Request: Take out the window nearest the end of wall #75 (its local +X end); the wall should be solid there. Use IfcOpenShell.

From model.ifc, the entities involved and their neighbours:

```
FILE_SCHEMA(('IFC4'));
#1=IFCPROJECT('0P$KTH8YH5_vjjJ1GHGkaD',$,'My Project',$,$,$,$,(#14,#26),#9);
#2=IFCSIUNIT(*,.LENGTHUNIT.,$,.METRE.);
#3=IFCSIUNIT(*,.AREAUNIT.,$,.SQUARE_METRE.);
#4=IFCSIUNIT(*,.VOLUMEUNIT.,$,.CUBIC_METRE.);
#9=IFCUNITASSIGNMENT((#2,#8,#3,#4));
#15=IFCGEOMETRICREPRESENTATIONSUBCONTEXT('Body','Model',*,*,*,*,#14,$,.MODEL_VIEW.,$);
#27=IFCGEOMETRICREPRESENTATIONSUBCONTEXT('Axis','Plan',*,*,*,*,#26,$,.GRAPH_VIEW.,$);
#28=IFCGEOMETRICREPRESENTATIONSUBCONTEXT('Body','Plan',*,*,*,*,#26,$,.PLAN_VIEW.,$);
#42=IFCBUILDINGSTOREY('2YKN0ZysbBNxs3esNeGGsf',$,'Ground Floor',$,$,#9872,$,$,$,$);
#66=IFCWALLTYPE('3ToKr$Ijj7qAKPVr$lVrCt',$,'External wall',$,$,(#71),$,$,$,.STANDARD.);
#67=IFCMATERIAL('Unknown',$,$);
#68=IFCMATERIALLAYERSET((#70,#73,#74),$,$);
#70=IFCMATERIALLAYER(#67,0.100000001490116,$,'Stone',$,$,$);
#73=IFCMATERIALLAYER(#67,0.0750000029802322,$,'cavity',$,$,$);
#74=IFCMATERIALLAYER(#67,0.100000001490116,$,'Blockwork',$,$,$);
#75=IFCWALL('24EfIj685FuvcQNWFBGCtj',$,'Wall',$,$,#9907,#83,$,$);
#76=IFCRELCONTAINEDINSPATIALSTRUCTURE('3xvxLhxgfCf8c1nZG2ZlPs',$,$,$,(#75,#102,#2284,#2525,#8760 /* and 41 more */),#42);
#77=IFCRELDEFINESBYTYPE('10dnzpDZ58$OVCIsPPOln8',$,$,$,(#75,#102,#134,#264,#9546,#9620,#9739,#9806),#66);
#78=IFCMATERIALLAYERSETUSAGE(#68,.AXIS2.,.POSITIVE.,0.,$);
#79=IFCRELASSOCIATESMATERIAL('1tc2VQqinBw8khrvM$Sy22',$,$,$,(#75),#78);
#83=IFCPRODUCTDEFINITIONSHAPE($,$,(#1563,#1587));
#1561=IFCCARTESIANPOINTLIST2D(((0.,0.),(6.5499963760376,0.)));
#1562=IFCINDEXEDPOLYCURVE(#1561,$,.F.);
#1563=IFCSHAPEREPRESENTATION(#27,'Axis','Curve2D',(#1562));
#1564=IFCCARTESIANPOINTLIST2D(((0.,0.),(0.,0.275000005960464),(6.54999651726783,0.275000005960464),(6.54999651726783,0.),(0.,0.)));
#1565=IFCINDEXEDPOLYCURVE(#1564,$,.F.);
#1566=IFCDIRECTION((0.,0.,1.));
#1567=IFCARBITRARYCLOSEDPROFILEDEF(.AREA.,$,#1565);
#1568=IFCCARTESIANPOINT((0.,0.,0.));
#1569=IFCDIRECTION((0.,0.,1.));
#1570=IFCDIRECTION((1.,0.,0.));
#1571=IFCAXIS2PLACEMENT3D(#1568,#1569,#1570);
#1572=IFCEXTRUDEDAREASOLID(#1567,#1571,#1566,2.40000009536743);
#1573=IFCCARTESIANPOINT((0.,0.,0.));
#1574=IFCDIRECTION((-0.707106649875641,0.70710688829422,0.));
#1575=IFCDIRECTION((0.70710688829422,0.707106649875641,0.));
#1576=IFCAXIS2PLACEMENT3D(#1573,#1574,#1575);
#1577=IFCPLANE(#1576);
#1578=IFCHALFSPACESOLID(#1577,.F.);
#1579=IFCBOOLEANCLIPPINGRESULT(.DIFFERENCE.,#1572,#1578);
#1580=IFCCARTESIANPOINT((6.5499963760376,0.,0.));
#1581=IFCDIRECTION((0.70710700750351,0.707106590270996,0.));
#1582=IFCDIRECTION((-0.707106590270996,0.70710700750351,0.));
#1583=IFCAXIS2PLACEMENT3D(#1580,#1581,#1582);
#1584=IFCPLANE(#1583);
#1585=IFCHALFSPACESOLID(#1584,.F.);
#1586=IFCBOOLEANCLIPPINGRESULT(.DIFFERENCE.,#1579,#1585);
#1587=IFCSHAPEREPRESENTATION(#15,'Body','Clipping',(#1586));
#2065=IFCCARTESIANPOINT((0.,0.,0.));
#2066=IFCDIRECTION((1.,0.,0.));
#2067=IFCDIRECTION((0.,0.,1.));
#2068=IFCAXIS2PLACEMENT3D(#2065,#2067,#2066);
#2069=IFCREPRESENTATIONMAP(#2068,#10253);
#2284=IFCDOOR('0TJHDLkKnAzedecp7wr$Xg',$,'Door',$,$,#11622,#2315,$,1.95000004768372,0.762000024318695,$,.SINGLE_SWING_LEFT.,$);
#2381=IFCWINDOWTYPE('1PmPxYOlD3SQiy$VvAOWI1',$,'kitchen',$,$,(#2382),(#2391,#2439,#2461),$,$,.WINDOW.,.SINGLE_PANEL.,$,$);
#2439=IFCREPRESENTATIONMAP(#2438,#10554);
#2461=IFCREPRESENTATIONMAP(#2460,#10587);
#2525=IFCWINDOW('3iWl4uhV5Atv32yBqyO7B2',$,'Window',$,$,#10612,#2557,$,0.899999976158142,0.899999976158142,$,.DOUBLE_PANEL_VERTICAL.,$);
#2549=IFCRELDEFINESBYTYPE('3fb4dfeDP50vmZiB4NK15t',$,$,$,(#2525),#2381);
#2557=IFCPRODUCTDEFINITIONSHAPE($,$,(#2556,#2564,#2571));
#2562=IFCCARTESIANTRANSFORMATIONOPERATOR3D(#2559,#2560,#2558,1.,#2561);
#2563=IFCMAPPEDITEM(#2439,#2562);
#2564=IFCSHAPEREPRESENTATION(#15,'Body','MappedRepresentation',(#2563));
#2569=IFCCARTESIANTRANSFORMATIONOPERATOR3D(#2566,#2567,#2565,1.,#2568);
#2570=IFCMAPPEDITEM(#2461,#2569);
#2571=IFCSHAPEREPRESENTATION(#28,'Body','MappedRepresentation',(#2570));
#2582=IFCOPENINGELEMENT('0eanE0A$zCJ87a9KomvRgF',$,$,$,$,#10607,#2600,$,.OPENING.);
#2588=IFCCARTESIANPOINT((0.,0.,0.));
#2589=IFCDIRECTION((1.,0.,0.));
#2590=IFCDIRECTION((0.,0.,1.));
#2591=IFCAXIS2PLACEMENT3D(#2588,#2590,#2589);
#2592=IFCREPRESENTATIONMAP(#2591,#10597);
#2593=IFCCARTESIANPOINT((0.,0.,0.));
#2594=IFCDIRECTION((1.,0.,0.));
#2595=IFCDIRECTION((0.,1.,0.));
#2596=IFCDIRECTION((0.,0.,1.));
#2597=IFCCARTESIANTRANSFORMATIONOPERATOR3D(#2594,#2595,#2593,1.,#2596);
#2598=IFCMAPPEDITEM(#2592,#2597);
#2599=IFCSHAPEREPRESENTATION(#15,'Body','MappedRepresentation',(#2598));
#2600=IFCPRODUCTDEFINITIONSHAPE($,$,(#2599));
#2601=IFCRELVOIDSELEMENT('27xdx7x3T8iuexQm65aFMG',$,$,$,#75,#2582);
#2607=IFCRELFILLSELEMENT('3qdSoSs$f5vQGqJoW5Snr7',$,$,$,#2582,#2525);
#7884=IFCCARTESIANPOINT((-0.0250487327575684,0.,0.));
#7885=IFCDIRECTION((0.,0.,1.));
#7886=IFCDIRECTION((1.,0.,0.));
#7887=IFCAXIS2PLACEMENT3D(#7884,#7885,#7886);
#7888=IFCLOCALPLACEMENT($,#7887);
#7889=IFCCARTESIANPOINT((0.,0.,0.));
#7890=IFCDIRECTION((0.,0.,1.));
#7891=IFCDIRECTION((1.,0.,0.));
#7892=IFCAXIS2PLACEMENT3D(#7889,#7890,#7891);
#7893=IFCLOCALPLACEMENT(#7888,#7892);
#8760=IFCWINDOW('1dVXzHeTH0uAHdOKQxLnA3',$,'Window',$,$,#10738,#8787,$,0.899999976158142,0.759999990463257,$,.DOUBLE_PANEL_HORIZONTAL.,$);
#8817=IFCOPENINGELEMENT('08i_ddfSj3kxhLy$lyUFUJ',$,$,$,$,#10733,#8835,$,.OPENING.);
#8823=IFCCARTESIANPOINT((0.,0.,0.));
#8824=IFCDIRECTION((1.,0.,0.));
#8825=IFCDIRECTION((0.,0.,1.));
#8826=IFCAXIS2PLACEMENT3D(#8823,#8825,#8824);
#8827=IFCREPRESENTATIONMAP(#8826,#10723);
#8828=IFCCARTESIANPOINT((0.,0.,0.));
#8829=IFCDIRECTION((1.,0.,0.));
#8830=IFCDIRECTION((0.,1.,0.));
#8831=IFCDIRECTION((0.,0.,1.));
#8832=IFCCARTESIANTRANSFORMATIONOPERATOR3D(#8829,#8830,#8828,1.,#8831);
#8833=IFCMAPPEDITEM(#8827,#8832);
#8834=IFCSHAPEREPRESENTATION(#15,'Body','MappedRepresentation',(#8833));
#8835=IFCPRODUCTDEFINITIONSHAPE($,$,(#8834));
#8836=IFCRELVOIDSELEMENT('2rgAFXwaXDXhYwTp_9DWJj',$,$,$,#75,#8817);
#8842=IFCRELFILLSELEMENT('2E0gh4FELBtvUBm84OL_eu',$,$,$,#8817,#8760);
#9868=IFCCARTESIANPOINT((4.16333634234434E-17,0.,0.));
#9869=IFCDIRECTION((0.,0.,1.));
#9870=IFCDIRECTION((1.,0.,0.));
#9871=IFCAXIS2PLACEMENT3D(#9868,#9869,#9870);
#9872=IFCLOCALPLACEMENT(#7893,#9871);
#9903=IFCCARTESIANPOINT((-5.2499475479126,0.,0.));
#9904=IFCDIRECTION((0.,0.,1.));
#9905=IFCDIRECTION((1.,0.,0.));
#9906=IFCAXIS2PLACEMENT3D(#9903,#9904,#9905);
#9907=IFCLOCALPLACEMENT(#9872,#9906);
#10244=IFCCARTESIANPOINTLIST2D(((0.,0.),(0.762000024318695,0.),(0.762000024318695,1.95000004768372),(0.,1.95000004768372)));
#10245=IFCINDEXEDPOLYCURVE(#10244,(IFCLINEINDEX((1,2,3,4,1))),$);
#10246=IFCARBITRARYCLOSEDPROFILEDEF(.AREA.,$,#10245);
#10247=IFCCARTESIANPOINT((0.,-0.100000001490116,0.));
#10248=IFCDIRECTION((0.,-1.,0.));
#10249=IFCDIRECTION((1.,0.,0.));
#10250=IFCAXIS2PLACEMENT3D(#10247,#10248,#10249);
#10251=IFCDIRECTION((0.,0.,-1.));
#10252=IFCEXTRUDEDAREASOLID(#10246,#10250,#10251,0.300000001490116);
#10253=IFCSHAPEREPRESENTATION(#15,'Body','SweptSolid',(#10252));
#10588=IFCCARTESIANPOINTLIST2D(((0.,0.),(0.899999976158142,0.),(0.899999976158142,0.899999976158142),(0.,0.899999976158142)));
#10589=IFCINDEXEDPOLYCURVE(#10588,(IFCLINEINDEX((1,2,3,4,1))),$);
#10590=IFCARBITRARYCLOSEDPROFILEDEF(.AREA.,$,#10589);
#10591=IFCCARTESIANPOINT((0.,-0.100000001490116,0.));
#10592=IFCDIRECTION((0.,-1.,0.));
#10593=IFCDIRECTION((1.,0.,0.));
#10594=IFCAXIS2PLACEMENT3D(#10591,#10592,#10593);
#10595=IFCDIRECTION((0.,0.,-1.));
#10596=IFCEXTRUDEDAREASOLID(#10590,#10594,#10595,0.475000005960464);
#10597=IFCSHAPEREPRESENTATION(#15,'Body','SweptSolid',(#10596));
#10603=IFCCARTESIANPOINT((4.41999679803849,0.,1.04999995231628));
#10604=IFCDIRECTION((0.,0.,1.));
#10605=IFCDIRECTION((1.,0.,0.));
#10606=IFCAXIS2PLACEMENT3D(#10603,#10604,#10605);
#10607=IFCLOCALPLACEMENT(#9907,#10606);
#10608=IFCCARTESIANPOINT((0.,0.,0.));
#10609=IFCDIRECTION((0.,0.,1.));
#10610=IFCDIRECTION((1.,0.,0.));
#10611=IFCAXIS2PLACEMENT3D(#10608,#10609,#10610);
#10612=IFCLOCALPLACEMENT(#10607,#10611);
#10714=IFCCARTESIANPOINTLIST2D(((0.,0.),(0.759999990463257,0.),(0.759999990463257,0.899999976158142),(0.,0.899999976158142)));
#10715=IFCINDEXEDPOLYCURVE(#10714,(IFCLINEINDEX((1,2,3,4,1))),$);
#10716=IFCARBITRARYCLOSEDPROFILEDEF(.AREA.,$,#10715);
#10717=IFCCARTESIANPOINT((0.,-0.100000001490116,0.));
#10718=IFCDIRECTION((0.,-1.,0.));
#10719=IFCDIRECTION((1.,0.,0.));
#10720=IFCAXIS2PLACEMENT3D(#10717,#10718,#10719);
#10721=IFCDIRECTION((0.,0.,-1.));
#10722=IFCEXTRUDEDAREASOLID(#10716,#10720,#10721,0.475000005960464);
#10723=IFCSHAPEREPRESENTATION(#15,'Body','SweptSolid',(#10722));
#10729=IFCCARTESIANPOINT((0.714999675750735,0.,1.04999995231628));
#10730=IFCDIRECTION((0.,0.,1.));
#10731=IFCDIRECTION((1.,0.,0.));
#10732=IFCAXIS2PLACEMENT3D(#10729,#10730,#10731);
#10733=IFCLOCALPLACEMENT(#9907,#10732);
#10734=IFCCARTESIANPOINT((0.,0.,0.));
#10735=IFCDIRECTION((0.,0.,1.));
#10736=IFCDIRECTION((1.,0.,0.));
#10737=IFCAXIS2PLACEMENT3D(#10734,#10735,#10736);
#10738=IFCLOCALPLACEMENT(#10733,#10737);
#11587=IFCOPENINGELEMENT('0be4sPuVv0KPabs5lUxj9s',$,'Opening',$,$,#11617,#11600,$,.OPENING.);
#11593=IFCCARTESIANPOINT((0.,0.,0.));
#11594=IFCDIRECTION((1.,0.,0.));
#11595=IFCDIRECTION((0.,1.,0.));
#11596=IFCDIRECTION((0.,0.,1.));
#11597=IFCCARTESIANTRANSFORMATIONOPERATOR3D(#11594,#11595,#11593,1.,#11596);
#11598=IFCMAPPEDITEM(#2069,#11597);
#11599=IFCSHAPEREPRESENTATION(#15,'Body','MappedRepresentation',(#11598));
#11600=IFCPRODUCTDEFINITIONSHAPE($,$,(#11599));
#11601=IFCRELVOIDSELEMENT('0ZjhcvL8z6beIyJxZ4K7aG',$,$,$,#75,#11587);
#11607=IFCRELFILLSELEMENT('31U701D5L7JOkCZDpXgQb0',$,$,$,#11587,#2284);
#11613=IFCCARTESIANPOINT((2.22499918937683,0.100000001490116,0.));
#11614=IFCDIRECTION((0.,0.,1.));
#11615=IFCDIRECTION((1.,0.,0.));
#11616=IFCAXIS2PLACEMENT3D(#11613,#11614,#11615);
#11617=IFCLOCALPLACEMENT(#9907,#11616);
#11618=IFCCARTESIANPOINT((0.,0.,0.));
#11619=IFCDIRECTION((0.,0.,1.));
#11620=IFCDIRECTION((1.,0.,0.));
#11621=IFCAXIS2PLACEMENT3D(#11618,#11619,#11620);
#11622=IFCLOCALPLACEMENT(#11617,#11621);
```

```python
import ifcopenshell
import ifcopenshell.api.feature
import ifcopenshell.api.root
import ifcopenshell.geom
import ifcopenshell.util.shape

model = ifcopenshell.open("model.ifc")
settings = ifcopenshell.geom.settings()


def volume(element):
    """Net volume in cubic metres, openings subtracted."""
    shape = ifcopenshell.geom.create_shape(settings, element)
    return ifcopenshell.util.shape.get_volume(shape.geometry)


window = model.by_guid("3iWl4uhV5Atv32yBqyO7B2")
opening = window.FillsVoids[0].RelatingOpeningElement
wall = opening.VoidsElements[0].RelatingBuildingElement
before = volume(wall)

ifcopenshell.api.root.remove_product(model, product=window)
ifcopenshell.api.feature.remove_feature(model, feature=opening)

after = volume(wall)

print(f"wall volume {before:.3f} -> {after:.3f} m3")

model.write("model_updated.ifc")
```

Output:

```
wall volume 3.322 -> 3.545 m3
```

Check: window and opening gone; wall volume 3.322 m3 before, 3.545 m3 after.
